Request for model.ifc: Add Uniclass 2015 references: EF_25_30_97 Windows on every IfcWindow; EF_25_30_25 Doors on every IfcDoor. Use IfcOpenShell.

First a look at what the model holds.

```python
import ifcopenshell

model = ifcopenshell.open("model.ifc")
print(model.schema)
print("classifications:", [c.Name for c in model.by_type("IfcClassification")])
for ifc_class in ("IfcDoor", "IfcRoof", "IfcStair", "IfcWall", "IfcWindow"):
    print(ifc_class, len(model.by_type(ifc_class)))
```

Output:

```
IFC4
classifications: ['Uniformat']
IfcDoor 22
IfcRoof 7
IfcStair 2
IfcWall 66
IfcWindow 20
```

```python
import ifcopenshell
import ifcopenshell.api.classification

model = ifcopenshell.open("model.ifc")

system = ifcopenshell.api.classification.add_classification(model, classification="Uniclass 2015")

codes = {
    "IfcWindow": ("EF_25_30_97", "Windows"),
    "IfcDoor": ("EF_25_30_25", "Doors"),
}
for ifc_class, (code, name) in codes.items():
    products = model.by_type(ifc_class)
    ifcopenshell.api.classification.add_reference(
        model, products=products, classification=system, identification=code, name=name
    )
    print(code, len(products))

model.write("model_edited.ifc")
```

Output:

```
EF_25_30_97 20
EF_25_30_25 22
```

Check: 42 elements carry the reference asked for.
